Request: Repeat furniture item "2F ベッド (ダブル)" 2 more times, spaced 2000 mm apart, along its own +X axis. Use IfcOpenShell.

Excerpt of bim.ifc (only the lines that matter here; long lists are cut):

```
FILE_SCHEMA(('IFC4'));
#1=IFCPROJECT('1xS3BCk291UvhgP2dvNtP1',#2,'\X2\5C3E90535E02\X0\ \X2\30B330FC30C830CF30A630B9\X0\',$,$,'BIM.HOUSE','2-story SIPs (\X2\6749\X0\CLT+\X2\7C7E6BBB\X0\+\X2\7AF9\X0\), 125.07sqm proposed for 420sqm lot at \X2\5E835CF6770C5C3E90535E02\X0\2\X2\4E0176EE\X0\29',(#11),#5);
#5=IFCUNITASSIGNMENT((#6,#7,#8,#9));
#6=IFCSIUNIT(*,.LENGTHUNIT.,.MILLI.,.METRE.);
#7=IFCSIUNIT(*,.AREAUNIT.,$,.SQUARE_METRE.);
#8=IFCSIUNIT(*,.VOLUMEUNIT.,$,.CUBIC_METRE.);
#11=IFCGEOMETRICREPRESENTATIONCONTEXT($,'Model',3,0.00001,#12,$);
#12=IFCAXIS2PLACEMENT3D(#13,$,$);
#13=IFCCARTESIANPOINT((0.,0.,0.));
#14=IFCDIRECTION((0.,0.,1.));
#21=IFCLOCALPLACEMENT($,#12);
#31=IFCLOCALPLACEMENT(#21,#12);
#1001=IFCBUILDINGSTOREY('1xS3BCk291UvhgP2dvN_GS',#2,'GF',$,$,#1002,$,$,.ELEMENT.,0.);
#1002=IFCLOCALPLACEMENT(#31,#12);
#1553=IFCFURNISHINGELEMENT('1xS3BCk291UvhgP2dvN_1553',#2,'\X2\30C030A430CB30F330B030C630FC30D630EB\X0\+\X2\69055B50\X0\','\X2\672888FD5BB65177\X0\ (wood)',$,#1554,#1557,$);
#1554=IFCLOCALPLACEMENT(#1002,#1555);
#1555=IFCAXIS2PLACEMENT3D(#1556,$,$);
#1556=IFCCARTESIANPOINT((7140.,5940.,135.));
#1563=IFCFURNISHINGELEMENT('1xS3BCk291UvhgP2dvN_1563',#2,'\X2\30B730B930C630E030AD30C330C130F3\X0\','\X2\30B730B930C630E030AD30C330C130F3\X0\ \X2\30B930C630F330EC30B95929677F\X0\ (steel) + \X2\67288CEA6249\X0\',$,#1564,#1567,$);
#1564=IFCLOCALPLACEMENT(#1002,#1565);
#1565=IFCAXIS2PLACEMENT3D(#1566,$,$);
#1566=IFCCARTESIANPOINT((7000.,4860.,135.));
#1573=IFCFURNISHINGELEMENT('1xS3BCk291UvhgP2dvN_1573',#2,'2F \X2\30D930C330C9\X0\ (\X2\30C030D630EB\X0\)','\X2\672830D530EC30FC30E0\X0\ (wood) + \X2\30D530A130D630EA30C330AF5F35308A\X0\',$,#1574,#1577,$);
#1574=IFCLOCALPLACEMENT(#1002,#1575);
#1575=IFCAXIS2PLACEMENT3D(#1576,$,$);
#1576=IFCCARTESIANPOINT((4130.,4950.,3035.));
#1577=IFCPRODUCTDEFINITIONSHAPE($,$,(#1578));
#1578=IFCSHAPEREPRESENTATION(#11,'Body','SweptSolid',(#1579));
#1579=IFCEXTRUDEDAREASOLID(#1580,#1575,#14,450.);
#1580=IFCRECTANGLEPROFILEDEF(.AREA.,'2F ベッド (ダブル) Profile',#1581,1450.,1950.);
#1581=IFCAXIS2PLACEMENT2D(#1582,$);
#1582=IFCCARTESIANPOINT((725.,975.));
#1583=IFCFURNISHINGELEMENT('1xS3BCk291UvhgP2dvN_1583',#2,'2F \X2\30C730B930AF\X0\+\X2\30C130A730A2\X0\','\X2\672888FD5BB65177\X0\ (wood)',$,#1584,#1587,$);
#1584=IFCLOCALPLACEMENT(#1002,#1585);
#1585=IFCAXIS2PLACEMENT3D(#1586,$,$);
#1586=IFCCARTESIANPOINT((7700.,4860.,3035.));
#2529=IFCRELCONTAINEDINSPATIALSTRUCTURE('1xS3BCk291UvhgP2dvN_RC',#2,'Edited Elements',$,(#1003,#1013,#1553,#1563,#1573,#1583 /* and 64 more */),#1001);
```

```python
import ifcopenshell
import ifcopenshell.api.geometry
import ifcopenshell.api.root
import ifcopenshell.util.element
import ifcopenshell.util.placement

model = ifcopenshell.open("bim.ifc")


def reuse_history(source, copy):
    """copy_class also copies each property set's owner history, people and application; keep the originals."""
    for rel in copy.IsDefinedBy:
        if rel.is_a("IfcRelDefinesByProperties") and (history := rel.RelatingPropertyDefinition.OwnerHistory):
            rel.RelatingPropertyDefinition.OwnerHistory = source.OwnerHistory
            ifcopenshell.util.element.remove_deep2(model, history)


source = model.by_guid("1xS3BCk291UvhgP2dvN_1573")
base = ifcopenshell.util.placement.get_local_placement(source.ObjectPlacement)
step = base[:3, 0] * 2000.0

for i in range(1, 3):
    copy = ifcopenshell.api.root.copy_class(model, product=source)
    copy.Representation = ifcopenshell.util.element.copy_deep(
        model, source.Representation, exclude=["IfcGeometricRepresentationContext", "IfcRepresentationMap"]
    )
    reuse_history(source, copy)
    matrix = base.copy()
    matrix[:3, 3] += i * step
    print("added at", matrix[:3, 3].round(3) + 0.0)
    ifcopenshell.api.geometry.edit_object_placement(model, product=copy, matrix=matrix, is_si=False)

model.write("bim_edited.ifc")
```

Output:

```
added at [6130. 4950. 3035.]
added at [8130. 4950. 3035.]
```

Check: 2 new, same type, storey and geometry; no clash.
